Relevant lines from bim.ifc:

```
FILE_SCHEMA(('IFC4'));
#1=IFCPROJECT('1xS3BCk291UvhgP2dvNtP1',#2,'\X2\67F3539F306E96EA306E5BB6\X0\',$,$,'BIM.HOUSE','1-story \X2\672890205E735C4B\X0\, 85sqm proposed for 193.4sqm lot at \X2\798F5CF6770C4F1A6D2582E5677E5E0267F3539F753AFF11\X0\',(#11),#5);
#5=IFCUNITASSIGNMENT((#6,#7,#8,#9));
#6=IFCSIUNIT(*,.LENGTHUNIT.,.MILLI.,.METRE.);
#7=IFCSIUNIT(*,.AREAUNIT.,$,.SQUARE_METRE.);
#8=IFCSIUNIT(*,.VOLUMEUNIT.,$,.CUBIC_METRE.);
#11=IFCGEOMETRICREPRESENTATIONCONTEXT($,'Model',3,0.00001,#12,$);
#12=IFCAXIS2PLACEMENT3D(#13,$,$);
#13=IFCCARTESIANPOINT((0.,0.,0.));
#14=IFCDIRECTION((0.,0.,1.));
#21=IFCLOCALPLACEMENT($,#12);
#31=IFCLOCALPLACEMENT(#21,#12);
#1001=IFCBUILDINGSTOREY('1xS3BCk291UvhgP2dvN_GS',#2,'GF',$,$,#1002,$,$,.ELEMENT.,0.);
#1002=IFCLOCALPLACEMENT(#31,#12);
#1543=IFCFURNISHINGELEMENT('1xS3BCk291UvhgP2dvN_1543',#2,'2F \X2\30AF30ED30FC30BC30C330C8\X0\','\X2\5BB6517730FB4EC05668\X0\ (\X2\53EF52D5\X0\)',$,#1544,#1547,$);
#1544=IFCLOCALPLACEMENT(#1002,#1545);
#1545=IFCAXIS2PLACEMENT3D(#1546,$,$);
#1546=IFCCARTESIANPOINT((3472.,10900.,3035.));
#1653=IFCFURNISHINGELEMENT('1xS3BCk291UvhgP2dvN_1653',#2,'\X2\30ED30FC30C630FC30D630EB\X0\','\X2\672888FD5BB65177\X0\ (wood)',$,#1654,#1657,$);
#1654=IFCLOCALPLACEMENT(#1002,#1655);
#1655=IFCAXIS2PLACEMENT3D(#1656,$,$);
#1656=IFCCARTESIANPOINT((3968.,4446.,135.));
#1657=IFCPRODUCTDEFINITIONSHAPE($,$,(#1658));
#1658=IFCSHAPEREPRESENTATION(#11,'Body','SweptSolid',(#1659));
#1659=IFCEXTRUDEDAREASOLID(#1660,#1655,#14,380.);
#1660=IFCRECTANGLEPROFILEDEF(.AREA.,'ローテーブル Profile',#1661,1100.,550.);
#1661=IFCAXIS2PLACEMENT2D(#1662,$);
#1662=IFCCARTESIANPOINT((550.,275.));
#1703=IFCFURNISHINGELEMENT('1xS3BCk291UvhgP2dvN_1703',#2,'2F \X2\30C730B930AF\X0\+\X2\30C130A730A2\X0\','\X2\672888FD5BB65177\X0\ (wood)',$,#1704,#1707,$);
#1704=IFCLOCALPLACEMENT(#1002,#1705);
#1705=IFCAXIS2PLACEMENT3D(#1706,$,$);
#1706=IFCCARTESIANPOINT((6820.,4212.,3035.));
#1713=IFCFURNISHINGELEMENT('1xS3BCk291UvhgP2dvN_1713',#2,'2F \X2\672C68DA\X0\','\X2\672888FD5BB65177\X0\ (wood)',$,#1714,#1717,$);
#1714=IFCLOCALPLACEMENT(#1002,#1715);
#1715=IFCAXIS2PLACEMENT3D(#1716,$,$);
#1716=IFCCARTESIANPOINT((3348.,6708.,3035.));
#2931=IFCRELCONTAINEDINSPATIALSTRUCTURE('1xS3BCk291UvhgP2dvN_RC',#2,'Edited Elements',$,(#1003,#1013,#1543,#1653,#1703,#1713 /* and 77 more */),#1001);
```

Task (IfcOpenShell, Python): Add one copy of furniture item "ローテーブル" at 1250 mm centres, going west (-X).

```python
import numpy as np
import ifcopenshell
import ifcopenshell.api.geometry
import ifcopenshell.api.root
import ifcopenshell.util.element
import ifcopenshell.util.placement
import ifcopenshell.util.unit

model = ifcopenshell.open("bim.ifc")
unit_scale = ifcopenshell.util.unit.calculate_unit_scale(model)


def reuse_history(source, copy):
    """copy_class also copies each property set's owner history, people and application; keep the originals."""
    for rel in copy.IsDefinedBy:
        if rel.is_a("IfcRelDefinesByProperties") and (history := rel.RelatingPropertyDefinition.OwnerHistory):
            rel.RelatingPropertyDefinition.OwnerHistory = source.OwnerHistory
            ifcopenshell.util.element.remove_deep2(model, history)


source = model.by_guid("1xS3BCk291UvhgP2dvN_1653")
base = ifcopenshell.util.placement.get_local_placement(source.ObjectPlacement)
step = np.array([-1.0, 0.0, 0.0]) * 1.25 / unit_scale

for i in range(1, 2):
    copy = ifcopenshell.api.root.copy_class(model, product=source)
    copy.Representation = ifcopenshell.util.element.copy_deep(
        model, source.Representation, exclude=["IfcGeometricRepresentationContext", "IfcRepresentationMap"]
    )
    reuse_history(source, copy)
    matrix = base.copy()
    matrix[:3, 3] += i * step
    print("added at", matrix[:3, 3].round(3) + 0.0)
    ifcopenshell.api.geometry.edit_object_placement(model, product=copy, matrix=matrix, is_si=False)

model.write("bim_rev.ifc")
```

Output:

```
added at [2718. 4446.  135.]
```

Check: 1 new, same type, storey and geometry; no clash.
